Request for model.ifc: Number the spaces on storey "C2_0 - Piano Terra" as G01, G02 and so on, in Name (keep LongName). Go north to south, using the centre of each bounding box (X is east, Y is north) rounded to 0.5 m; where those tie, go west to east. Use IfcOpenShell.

First a look at what the model holds.

```python
import ifcopenshell
import ifcopenshell.util.element
import ifcopenshell.util.placement

model = ifcopenshell.open("model.ifc")
print(model.schema)
storey = next(s for s in model.by_type("IfcBuildingStorey") if s.Name == "C2_0 - Piano Terra")
spaces = [e for e in ifcopenshell.util.element.get_decomposition(storey) if e.is_a("IfcSpace")]
for e in sorted(spaces, key=lambda e: e.id()):
    origin = ifcopenshell.util.placement.get_local_placement(e.ObjectPlacement)[:3, 3]
    print(e.id(), e.Name, e.LongName, origin.round(2) + 0.0, sep=" | ")
```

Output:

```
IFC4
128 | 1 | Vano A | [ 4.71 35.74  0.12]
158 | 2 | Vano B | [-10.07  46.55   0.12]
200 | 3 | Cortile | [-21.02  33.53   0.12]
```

```python
import ifcopenshell
import ifcopenshell.geom
import ifcopenshell.util.element
import ifcopenshell.util.shape

model = ifcopenshell.open("model.ifc")
settings = ifcopenshell.geom.settings()
settings.set("use-world-coords", True)


def centre(element):
    shape = ifcopenshell.geom.create_shape(settings, element)
    return ifcopenshell.util.shape.get_bbox_centroid(shape.geometry)


storey = next(s for s in model.by_type("IfcBuildingStorey") if s.Name == "C2_0 - Piano Terra")
spaces = [e for e in ifcopenshell.util.element.get_decomposition(storey) if e.is_a("IfcSpace")]

# Insertion points can sit at a corner or the storey origin, so sort by the geometry (in metres).
centres = {e: centre(e) for e in spaces}
spaces.sort(key=lambda e: (-round(centres[e][1] / 0.5), centres[e][0]))

for i, e in enumerate(spaces, start=1):
    number = f"G{i:02d}"
    e.Name = number
    print(e.id(), number)

model.write("model-out.ifc")
```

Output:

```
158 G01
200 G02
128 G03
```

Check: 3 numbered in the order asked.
